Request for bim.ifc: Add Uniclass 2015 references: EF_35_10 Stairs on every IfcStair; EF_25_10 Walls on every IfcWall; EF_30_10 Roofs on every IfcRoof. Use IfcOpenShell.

First a look at what the model holds.

```python
import ifcopenshell

model = ifcopenshell.open("bim.ifc")
print(model.schema)
print("classifications:", [c.Name for c in model.by_type("IfcClassification")])
for ifc_class in ("IfcDoor", "IfcRoof", "IfcStair", "IfcWall", "IfcWindow"):
    print(ifc_class, len(model.by_type(ifc_class)))
```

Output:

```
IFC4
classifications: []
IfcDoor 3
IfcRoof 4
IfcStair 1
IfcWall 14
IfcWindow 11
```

```python
import ifcopenshell
import ifcopenshell.api.classification

model = ifcopenshell.open("bim.ifc")

system = ifcopenshell.api.classification.add_classification(model, classification="Uniclass 2015")

codes = {
    "IfcStair": ("EF_35_10", "Stairs"),
    "IfcWall": ("EF_25_10", "Walls"),
    "IfcRoof": ("EF_30_10", "Roofs"),
}
for ifc_class, (code, name) in codes.items():
    products = model.by_type(ifc_class)
    ifcopenshell.api.classification.add_reference(
        model, products=products, classification=system, identification=code, name=name
    )
    print(code, len(products))

model.write("bim-out.ifc")
```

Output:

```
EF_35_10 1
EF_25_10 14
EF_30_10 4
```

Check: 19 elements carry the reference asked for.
